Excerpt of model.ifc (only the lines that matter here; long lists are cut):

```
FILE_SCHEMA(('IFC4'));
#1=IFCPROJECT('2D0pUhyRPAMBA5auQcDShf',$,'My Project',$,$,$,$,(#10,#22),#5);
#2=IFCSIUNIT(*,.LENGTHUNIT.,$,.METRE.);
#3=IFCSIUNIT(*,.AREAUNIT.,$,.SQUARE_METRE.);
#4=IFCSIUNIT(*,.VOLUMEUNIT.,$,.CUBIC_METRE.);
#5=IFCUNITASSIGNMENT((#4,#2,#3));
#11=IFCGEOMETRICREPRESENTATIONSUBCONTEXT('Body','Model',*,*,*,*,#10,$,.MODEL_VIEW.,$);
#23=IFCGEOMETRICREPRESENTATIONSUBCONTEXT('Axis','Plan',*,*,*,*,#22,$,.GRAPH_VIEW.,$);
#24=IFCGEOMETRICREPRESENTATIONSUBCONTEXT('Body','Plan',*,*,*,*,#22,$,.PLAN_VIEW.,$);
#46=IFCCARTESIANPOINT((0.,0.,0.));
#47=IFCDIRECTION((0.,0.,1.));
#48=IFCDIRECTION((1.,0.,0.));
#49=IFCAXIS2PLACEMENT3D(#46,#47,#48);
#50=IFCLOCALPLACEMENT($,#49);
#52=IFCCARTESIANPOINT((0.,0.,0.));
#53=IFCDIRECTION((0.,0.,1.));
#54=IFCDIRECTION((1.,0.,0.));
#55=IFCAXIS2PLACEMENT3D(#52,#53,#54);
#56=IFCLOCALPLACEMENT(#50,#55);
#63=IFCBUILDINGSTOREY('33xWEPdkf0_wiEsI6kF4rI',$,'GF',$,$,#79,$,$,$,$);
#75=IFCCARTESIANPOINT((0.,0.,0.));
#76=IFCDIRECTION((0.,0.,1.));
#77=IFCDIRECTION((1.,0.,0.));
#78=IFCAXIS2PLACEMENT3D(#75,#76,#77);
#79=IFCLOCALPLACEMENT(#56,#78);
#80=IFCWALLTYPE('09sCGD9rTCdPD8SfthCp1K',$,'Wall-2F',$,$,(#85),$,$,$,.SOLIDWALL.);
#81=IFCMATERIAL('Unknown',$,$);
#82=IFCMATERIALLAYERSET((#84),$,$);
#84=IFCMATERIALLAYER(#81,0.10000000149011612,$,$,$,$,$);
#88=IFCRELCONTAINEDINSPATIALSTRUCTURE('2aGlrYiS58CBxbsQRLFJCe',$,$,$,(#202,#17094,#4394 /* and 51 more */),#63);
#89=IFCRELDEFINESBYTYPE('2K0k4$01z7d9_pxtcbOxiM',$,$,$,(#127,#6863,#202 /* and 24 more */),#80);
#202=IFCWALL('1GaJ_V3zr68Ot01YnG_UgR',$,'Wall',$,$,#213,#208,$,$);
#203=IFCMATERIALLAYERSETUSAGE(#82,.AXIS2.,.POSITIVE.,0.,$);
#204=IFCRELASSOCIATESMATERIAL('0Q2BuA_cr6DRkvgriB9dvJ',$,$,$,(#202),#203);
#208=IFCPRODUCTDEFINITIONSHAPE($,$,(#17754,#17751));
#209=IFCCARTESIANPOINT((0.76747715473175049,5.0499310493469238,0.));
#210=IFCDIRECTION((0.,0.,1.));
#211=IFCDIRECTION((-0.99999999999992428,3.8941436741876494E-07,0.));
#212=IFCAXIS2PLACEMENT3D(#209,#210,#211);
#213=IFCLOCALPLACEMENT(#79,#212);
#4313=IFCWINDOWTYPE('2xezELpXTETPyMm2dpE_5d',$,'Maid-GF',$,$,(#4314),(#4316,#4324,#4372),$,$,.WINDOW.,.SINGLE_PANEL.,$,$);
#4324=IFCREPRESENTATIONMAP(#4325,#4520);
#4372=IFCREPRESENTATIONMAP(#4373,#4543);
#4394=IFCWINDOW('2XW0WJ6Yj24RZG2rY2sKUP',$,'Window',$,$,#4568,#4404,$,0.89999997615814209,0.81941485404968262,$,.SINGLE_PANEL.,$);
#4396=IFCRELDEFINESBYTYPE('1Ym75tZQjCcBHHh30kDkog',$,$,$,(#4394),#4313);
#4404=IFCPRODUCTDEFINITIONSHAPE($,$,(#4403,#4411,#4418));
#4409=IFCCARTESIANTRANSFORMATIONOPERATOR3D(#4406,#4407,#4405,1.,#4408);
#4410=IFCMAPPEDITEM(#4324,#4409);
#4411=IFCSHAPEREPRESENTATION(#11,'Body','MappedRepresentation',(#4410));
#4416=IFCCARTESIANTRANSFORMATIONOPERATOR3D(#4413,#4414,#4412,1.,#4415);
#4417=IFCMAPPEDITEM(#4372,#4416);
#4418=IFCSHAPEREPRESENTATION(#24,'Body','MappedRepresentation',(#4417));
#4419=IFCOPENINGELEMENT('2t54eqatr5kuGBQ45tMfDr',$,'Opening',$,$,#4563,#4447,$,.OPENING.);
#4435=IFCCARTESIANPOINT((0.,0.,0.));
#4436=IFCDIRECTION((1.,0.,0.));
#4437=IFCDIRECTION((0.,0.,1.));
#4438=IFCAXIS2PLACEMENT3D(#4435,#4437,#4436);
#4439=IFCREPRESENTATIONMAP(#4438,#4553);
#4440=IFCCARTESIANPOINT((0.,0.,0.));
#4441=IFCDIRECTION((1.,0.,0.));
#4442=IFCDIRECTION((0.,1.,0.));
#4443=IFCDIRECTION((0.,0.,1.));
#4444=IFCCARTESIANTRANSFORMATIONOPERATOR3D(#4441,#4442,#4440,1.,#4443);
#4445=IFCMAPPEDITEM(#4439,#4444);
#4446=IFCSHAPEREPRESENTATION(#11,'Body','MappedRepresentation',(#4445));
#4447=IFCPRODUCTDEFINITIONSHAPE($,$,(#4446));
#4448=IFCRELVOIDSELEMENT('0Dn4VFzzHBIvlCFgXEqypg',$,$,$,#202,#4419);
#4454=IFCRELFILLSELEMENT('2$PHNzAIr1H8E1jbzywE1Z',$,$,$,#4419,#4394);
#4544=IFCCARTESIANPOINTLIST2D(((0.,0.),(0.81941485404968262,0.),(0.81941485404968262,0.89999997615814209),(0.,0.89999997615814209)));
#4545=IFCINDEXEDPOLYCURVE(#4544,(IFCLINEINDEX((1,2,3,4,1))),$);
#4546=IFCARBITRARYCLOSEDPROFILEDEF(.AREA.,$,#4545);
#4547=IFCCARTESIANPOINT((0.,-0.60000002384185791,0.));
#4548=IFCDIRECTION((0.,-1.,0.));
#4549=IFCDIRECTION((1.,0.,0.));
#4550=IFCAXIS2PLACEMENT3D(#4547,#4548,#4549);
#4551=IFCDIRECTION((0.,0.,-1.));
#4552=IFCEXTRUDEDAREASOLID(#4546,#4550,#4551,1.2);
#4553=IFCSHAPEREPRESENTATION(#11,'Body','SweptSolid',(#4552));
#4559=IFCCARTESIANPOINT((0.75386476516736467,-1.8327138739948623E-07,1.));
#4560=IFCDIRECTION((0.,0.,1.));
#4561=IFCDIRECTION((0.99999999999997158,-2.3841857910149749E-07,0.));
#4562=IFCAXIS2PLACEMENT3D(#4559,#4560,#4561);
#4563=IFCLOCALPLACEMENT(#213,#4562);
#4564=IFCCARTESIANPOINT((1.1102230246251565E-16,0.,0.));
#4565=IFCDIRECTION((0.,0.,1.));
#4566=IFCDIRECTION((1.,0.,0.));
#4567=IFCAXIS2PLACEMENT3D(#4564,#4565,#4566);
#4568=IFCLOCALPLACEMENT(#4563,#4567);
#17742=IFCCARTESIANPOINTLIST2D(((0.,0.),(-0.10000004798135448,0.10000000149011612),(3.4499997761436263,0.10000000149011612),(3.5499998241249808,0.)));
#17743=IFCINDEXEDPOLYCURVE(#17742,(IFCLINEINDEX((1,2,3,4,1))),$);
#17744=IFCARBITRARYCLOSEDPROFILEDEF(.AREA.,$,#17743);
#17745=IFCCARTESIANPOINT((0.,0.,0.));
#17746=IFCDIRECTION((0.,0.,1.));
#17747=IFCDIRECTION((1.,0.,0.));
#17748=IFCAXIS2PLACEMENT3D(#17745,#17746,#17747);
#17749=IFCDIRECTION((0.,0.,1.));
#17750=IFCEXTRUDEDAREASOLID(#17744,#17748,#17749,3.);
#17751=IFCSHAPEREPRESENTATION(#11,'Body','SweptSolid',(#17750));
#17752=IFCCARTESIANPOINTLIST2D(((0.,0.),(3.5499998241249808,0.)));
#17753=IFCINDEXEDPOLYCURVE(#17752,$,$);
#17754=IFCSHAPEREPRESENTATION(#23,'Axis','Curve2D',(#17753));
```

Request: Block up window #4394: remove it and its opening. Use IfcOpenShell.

```python
import ifcopenshell
import ifcopenshell.api.feature
import ifcopenshell.api.root
import ifcopenshell.geom
import ifcopenshell.util.shape

model = ifcopenshell.open("model.ifc")
settings = ifcopenshell.geom.settings()


def volume(element):
    """Net volume in cubic metres, openings subtracted."""
    shape = ifcopenshell.geom.create_shape(settings, element)
    return ifcopenshell.util.shape.get_volume(shape.geometry)


window = model.by_id(4394)
opening = window.FillsVoids[0].RelatingOpeningElement
wall = opening.VoidsElements[0].RelatingBuildingElement
before = volume(wall)

ifcopenshell.api.root.remove_product(model, product=window)
ifcopenshell.api.feature.remove_feature(model, feature=opening)

after = volume(wall)

print(f"wall volume {before:.3f} -> {after:.3f} m3")

model.write("model_updated.ifc")
```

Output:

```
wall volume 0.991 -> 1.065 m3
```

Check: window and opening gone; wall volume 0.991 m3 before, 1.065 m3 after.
